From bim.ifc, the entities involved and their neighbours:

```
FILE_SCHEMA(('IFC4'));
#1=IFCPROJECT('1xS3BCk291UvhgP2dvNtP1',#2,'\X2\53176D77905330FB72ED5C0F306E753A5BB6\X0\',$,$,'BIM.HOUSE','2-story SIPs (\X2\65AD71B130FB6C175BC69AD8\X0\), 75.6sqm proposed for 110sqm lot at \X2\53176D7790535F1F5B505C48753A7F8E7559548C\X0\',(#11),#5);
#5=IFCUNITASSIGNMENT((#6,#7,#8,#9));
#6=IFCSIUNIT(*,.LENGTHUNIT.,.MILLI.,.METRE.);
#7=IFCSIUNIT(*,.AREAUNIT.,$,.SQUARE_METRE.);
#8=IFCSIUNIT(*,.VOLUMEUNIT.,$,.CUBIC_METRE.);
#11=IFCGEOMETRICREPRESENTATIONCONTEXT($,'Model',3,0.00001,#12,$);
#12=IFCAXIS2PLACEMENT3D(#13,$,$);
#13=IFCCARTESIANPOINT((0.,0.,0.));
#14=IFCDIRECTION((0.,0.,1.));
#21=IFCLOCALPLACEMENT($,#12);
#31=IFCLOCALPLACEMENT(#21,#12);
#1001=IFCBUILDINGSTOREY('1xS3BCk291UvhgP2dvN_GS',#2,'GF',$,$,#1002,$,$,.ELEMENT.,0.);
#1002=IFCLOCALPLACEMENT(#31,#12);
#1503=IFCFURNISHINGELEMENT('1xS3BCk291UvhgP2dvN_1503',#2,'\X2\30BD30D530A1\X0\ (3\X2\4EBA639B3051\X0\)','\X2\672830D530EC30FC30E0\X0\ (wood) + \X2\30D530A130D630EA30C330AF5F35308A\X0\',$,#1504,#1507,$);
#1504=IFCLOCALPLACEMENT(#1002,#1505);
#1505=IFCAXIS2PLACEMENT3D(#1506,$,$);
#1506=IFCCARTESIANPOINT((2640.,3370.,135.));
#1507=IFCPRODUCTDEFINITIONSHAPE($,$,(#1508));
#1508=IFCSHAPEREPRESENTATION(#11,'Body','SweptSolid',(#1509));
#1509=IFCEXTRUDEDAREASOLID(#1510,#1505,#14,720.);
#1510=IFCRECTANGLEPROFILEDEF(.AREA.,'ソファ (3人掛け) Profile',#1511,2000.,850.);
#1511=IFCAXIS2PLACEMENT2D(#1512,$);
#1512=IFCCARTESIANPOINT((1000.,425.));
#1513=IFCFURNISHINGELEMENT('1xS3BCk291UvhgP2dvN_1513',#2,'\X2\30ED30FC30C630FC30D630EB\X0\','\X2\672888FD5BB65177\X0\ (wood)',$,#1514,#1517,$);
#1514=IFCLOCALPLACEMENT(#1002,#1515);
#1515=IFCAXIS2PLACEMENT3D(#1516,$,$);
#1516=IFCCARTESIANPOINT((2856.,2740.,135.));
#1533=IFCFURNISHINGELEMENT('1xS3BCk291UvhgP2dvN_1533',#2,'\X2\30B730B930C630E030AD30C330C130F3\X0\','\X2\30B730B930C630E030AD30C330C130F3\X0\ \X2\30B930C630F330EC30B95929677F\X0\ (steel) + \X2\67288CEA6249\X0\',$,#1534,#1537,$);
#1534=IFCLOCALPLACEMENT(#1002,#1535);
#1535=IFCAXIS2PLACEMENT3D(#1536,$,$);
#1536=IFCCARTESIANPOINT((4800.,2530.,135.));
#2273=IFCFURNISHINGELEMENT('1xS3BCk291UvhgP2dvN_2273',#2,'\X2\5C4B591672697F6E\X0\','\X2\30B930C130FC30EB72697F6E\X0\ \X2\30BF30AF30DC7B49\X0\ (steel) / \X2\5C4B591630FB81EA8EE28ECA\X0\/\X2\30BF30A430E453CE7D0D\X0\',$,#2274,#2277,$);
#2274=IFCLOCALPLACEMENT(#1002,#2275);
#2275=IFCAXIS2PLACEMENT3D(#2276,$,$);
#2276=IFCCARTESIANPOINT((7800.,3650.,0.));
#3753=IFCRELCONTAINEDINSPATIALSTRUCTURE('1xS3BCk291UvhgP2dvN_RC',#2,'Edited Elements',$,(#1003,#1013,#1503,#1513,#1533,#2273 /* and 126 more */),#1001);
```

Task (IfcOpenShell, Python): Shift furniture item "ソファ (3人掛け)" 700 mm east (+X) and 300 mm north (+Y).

```python
import ifcopenshell
import ifcopenshell.api.geometry
import ifcopenshell.util.placement
import ifcopenshell.util.unit

model = ifcopenshell.open("bim.ifc")
unit_scale = ifcopenshell.util.unit.calculate_unit_scale(model)

item = model.by_guid("1xS3BCk291UvhgP2dvN_1503")
matrix = ifcopenshell.util.placement.get_local_placement(item.ObjectPlacement)
matrix[0, 3] += 0.7 / unit_scale
matrix[1, 3] += 0.3 / unit_scale
ifcopenshell.api.geometry.edit_object_placement(model, product=item, matrix=matrix, is_si=False)

print(ifcopenshell.util.placement.get_local_placement(item.ObjectPlacement).round(3) + 0.0)

model.write("bim-out.ifc")
```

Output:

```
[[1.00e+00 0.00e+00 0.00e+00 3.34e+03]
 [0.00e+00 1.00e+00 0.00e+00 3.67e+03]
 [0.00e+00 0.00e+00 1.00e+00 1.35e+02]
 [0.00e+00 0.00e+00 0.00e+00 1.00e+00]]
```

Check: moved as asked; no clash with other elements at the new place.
